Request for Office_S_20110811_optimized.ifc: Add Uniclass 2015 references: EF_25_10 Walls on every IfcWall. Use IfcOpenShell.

First a look at what the model holds.

```python
import ifcopenshell

model = ifcopenshell.open("Office_S_20110811_optimized.ifc")
print(model.schema)
print("classifications:", [c.Name for c in model.by_type("IfcClassification")])
for ifc_class in ("IfcDoor", "IfcRoof", "IfcStair", "IfcWall", "IfcWindow"):
    print(ifc_class, len(model.by_type(ifc_class)))
```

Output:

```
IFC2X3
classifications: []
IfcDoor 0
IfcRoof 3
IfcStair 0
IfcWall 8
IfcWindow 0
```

```python
import ifcopenshell
import ifcopenshell.api.classification

model = ifcopenshell.open("Office_S_20110811_optimized.ifc")

# IFC2X3 requires Source and Edition and has no link from the project to the system.
system = model.create_entity("IfcClassification", Source="NBS", Edition="2015", Name="Uniclass 2015")

codes = {
    "IfcWall": ("EF_25_10", "Walls"),
}
for ifc_class, (code, name) in codes.items():
    products = model.by_type(ifc_class)
    ifcopenshell.api.classification.add_reference(
        model, products=products, classification=system, identification=code, name=name
    )
    print(code, len(products))

model.write("Office_S_20110811_optimized_rev.ifc")
```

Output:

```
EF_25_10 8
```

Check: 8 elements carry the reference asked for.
